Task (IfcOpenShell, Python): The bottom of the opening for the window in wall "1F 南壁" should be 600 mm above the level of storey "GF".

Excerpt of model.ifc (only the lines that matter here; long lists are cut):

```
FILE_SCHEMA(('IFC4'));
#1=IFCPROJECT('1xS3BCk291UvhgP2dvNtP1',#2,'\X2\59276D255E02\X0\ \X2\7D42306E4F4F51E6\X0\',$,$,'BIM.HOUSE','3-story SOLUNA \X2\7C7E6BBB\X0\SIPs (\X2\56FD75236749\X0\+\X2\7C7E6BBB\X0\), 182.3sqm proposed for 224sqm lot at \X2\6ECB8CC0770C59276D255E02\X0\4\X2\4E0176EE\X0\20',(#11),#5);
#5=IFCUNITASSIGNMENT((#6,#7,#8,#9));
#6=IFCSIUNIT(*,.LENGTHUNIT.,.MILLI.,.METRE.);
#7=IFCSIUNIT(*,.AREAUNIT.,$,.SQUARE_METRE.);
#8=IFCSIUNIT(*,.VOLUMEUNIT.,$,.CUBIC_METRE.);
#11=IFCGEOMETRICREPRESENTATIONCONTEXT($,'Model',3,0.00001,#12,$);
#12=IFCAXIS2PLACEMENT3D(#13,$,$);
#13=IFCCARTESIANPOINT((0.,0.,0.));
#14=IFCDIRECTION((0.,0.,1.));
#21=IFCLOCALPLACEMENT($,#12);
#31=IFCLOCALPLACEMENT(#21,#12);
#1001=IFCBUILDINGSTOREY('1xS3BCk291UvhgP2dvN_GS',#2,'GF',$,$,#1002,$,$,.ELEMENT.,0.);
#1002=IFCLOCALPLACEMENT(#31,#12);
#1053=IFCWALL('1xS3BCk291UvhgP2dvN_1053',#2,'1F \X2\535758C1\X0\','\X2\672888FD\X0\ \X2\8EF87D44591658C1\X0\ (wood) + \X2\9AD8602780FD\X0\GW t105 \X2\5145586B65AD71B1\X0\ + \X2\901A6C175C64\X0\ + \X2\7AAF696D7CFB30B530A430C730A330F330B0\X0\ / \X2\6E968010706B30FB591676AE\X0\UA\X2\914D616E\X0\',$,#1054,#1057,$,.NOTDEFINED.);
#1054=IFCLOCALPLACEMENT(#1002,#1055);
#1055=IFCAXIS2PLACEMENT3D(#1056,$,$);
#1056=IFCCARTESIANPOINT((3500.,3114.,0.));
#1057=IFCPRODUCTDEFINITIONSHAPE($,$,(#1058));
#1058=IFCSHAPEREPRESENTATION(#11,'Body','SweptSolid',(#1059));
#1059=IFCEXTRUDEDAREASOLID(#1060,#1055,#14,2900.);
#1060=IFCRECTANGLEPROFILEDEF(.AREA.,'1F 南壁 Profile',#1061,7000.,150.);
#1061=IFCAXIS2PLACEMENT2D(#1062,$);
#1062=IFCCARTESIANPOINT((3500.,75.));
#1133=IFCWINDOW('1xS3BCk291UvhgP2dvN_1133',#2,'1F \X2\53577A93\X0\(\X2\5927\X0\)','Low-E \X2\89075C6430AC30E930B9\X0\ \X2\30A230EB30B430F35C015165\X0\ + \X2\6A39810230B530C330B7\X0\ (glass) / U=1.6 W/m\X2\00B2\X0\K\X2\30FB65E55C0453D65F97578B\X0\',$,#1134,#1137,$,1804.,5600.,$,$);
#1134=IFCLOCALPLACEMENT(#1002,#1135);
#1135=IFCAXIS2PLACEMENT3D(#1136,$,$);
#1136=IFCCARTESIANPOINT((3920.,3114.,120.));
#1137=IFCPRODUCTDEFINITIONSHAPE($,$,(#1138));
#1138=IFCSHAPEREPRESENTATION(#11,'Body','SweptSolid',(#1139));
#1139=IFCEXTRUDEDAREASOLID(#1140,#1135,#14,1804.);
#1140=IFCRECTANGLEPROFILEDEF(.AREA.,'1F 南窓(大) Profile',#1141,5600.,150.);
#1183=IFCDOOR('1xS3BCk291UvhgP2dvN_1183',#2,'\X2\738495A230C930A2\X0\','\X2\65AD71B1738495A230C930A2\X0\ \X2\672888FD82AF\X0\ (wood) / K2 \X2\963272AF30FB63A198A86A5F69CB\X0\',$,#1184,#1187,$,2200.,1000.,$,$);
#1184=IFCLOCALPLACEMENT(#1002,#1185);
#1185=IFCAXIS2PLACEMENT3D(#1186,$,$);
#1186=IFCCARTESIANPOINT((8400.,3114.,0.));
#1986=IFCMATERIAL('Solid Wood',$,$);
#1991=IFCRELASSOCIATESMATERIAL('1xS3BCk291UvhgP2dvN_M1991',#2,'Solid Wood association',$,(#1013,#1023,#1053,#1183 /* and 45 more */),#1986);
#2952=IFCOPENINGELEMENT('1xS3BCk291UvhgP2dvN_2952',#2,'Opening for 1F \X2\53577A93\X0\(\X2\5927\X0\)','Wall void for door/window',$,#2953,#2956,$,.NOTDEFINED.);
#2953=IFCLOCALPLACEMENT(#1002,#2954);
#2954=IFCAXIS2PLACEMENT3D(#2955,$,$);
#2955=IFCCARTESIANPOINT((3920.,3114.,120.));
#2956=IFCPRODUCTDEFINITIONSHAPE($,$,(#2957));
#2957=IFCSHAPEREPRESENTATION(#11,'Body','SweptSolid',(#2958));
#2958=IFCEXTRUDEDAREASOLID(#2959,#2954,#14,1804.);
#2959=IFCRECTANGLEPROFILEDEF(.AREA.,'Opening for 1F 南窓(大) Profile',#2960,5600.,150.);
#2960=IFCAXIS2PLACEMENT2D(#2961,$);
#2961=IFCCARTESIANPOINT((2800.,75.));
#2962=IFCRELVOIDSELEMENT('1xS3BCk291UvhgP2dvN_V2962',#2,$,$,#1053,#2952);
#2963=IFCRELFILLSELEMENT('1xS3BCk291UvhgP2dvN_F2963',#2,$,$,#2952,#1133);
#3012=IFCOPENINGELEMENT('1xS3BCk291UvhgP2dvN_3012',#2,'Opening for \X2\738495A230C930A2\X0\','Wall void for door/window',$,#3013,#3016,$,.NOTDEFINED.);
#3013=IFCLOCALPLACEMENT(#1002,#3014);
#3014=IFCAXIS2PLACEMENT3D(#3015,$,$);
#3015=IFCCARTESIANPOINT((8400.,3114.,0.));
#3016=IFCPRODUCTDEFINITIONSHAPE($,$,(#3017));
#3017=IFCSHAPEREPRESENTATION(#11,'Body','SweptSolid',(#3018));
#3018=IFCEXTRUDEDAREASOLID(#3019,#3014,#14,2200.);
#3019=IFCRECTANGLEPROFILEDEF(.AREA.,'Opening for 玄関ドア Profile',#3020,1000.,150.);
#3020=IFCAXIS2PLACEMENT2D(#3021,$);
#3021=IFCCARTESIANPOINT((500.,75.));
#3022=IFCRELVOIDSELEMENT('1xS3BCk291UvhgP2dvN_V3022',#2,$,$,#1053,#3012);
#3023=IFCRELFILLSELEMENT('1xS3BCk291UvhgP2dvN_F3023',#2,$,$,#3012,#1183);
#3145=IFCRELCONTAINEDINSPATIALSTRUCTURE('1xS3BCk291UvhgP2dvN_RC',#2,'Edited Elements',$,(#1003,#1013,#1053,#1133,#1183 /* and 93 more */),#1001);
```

```python
import numpy as np
import ifcopenshell
import ifcopenshell.api.geometry
import ifcopenshell.geom
import ifcopenshell.util.element
import ifcopenshell.util.placement
import ifcopenshell.util.shape
import ifcopenshell.util.unit

model = ifcopenshell.open("model.ifc")
unit_scale = ifcopenshell.util.unit.calculate_unit_scale(model)

window = model.by_guid("1xS3BCk291UvhgP2dvN_1133")
opening = window.FillsVoids[0].RelatingOpeningElement
storey = ifcopenshell.util.element.get_container(window, ifc_class="IfcBuildingStorey")
level = ifcopenshell.util.placement.get_local_placement(storey.ObjectPlacement)[2, 3]

# The opening's origin need not be at the sill, so measure its lowest point.
shape = ifcopenshell.geom.create_shape(ifcopenshell.geom.settings(), opening)
bottom = ifcopenshell.util.shape.get_shape_bottom_elevation(shape, shape.geometry) / unit_scale
dz = level + 0.6 / unit_scale - bottom

shift = np.array([0.0, 0.0, dz])
# The window is not placed relative to its opening, so move both.
for product in (opening, window):
    matrix = ifcopenshell.util.placement.get_local_placement(product.ObjectPlacement)
    matrix[:3, 3] += shift
    ifcopenshell.api.geometry.edit_object_placement(model, product=product, matrix=matrix, is_si=False)

print(f"moved by {dz * unit_scale:+.3f} m")

model.write("model_rev.ifc")
```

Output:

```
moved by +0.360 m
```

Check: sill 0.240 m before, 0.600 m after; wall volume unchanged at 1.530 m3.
